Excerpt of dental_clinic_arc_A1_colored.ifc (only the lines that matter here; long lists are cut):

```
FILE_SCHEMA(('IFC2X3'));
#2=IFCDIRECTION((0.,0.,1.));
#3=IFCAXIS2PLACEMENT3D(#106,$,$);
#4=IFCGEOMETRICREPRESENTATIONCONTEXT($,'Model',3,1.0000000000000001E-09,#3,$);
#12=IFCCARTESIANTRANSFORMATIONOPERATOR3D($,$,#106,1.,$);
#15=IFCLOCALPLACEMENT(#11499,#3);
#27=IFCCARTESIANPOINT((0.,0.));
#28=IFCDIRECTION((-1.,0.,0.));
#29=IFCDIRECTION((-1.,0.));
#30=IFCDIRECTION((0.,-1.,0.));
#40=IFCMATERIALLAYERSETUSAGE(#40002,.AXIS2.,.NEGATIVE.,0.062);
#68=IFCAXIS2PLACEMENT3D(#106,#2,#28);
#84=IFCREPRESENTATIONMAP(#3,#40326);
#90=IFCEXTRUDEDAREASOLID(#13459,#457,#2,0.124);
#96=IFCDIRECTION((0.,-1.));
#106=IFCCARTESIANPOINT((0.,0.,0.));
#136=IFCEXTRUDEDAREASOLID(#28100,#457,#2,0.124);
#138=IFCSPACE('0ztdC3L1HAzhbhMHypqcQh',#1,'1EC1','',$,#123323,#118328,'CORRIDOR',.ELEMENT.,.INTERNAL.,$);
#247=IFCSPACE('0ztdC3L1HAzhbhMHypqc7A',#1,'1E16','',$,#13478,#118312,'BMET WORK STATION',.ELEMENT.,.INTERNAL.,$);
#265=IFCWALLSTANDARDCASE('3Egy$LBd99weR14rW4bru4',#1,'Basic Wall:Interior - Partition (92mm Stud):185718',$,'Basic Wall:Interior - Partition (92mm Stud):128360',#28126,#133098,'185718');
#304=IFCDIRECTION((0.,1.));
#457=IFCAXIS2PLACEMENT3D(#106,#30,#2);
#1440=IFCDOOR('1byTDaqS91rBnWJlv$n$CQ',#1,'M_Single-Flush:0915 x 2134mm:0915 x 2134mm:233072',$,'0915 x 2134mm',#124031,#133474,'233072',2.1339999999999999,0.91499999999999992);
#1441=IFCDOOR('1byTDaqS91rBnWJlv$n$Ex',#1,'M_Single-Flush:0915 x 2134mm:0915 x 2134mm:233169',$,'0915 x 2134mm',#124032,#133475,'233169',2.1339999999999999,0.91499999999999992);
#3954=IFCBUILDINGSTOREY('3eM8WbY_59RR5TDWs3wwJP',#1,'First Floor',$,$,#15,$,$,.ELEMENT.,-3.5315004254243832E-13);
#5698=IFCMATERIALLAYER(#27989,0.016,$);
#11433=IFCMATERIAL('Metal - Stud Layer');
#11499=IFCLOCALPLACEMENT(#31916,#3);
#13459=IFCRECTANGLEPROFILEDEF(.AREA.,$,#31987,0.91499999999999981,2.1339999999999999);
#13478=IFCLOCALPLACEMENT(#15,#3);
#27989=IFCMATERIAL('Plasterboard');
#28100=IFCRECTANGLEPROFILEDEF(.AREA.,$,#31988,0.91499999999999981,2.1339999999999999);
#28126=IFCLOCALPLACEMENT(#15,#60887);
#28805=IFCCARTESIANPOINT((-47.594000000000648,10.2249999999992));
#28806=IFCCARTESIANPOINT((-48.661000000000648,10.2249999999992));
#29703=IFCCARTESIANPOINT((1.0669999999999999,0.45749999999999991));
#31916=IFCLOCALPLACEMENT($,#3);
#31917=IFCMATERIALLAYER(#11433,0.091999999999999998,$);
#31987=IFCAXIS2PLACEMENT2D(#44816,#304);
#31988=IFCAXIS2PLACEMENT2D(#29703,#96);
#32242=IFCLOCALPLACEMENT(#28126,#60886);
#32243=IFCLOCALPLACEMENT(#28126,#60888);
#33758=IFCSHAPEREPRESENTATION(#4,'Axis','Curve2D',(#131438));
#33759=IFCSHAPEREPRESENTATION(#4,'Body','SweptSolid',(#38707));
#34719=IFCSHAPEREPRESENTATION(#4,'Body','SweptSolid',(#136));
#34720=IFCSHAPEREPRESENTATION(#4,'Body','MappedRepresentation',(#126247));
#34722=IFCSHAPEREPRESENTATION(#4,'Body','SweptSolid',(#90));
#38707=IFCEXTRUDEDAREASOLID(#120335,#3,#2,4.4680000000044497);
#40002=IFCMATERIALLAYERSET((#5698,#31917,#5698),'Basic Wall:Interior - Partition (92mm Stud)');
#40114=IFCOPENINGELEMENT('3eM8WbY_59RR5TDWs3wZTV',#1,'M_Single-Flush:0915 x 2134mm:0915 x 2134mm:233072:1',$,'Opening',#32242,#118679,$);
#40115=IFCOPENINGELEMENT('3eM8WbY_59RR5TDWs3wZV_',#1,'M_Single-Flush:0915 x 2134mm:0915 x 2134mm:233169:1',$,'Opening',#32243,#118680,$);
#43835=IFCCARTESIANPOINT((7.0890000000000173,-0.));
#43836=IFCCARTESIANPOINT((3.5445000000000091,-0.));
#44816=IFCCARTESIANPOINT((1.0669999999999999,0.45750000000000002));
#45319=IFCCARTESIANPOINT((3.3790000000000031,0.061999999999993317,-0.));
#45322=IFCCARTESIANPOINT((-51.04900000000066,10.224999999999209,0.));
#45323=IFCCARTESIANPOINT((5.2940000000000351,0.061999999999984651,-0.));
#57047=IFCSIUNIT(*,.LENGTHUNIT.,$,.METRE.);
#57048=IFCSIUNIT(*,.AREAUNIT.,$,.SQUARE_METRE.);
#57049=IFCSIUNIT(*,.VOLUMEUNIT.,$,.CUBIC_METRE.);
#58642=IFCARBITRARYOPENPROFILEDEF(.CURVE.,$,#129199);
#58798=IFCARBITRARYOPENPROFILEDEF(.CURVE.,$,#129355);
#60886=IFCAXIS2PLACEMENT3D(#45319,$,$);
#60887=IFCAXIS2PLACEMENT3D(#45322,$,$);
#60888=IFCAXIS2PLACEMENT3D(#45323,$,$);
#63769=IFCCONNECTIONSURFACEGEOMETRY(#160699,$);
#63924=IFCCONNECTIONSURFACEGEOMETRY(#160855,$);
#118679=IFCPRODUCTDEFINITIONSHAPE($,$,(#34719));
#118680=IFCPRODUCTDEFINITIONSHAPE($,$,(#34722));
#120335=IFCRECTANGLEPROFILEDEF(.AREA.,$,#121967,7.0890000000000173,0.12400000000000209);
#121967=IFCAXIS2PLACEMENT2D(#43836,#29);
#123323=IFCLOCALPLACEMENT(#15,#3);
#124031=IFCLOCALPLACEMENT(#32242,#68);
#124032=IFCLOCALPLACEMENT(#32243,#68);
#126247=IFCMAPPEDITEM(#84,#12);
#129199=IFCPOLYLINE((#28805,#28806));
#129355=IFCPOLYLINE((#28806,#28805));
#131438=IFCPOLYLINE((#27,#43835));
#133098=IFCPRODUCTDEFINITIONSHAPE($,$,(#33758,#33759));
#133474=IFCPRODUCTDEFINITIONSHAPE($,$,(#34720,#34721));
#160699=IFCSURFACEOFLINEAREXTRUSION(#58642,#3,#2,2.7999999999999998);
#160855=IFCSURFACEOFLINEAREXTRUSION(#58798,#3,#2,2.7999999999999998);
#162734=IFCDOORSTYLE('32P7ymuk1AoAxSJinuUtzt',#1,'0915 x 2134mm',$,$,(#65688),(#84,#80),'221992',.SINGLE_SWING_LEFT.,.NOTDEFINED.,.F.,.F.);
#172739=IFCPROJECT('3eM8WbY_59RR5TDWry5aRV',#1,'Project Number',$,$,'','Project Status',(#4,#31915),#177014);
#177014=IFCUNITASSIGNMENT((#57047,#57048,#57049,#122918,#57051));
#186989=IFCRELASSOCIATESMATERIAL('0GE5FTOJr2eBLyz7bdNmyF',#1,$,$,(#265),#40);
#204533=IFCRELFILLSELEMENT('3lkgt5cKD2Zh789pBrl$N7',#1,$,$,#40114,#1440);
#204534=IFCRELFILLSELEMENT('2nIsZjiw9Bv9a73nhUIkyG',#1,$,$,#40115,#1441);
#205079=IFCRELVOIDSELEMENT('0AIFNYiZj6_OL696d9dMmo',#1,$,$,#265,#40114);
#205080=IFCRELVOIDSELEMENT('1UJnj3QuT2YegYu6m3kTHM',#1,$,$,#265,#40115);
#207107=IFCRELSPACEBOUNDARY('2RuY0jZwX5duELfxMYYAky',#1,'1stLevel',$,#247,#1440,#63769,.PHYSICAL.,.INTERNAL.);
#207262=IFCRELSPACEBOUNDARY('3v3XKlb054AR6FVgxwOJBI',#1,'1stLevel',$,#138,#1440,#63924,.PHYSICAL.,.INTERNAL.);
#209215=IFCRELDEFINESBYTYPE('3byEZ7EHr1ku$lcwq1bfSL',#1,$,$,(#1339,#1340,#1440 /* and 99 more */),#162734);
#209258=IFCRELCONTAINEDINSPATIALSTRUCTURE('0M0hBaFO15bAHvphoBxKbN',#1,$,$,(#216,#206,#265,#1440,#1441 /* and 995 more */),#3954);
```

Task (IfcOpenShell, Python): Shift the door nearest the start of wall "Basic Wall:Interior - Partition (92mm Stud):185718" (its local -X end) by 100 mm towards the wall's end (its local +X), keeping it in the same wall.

```python
import numpy as np
import ifcopenshell
import ifcopenshell.api.geometry
import ifcopenshell.util.placement
import ifcopenshell.util.unit

model = ifcopenshell.open("dental_clinic_arc_A1_colored.ifc")
unit_scale = ifcopenshell.util.unit.calculate_unit_scale(model)

door = model.by_id(1440)
opening = door.FillsVoids[0].RelatingOpeningElement
wall = opening.VoidsElements[0].RelatingBuildingElement

wall_matrix = ifcopenshell.util.placement.get_local_placement(wall.ObjectPlacement)
shift = wall_matrix[:3, 0] * 0.1 / unit_scale
before = ifcopenshell.util.placement.get_local_placement(door.ObjectPlacement)[:3, 3].copy()

# The door is placed relative to its opening, so it follows when the opening moves.
matrix = ifcopenshell.util.placement.get_local_placement(opening.ObjectPlacement)
matrix[:3, 3] += shift
ifcopenshell.api.geometry.edit_object_placement(
    model, product=opening, matrix=matrix, is_si=False, should_transform_children=True
)

# Space boundary surfaces are stored in each space's coordinates; move them too.
for rel in door.ProvidesBoundaries:
    if not rel.ConnectionGeometry:
        continue
    surface = rel.ConnectionGeometry.SurfaceOnRelatingElement
    space_matrix = ifcopenshell.util.placement.get_local_placement(rel.RelatingSpace.ObjectPlacement)
    point = np.array(surface.Position.Location.Coordinates) + space_matrix[:3, :3].T @ shift
    surface.Position = model.createIfcAxis2Placement3D(
        model.createIfcCartesianPoint(point.tolist()), surface.Position.Axis, surface.Position.RefDirection
    )

after = ifcopenshell.util.placement.get_local_placement(door.ObjectPlacement)[:3, 3]
print("door moved by", (after - before).round(3) + 0.0)

model.write("dental_clinic_arc_A1_colored_rev.ifc")
```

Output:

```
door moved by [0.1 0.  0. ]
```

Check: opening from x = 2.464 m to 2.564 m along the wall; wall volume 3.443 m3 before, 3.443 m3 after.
